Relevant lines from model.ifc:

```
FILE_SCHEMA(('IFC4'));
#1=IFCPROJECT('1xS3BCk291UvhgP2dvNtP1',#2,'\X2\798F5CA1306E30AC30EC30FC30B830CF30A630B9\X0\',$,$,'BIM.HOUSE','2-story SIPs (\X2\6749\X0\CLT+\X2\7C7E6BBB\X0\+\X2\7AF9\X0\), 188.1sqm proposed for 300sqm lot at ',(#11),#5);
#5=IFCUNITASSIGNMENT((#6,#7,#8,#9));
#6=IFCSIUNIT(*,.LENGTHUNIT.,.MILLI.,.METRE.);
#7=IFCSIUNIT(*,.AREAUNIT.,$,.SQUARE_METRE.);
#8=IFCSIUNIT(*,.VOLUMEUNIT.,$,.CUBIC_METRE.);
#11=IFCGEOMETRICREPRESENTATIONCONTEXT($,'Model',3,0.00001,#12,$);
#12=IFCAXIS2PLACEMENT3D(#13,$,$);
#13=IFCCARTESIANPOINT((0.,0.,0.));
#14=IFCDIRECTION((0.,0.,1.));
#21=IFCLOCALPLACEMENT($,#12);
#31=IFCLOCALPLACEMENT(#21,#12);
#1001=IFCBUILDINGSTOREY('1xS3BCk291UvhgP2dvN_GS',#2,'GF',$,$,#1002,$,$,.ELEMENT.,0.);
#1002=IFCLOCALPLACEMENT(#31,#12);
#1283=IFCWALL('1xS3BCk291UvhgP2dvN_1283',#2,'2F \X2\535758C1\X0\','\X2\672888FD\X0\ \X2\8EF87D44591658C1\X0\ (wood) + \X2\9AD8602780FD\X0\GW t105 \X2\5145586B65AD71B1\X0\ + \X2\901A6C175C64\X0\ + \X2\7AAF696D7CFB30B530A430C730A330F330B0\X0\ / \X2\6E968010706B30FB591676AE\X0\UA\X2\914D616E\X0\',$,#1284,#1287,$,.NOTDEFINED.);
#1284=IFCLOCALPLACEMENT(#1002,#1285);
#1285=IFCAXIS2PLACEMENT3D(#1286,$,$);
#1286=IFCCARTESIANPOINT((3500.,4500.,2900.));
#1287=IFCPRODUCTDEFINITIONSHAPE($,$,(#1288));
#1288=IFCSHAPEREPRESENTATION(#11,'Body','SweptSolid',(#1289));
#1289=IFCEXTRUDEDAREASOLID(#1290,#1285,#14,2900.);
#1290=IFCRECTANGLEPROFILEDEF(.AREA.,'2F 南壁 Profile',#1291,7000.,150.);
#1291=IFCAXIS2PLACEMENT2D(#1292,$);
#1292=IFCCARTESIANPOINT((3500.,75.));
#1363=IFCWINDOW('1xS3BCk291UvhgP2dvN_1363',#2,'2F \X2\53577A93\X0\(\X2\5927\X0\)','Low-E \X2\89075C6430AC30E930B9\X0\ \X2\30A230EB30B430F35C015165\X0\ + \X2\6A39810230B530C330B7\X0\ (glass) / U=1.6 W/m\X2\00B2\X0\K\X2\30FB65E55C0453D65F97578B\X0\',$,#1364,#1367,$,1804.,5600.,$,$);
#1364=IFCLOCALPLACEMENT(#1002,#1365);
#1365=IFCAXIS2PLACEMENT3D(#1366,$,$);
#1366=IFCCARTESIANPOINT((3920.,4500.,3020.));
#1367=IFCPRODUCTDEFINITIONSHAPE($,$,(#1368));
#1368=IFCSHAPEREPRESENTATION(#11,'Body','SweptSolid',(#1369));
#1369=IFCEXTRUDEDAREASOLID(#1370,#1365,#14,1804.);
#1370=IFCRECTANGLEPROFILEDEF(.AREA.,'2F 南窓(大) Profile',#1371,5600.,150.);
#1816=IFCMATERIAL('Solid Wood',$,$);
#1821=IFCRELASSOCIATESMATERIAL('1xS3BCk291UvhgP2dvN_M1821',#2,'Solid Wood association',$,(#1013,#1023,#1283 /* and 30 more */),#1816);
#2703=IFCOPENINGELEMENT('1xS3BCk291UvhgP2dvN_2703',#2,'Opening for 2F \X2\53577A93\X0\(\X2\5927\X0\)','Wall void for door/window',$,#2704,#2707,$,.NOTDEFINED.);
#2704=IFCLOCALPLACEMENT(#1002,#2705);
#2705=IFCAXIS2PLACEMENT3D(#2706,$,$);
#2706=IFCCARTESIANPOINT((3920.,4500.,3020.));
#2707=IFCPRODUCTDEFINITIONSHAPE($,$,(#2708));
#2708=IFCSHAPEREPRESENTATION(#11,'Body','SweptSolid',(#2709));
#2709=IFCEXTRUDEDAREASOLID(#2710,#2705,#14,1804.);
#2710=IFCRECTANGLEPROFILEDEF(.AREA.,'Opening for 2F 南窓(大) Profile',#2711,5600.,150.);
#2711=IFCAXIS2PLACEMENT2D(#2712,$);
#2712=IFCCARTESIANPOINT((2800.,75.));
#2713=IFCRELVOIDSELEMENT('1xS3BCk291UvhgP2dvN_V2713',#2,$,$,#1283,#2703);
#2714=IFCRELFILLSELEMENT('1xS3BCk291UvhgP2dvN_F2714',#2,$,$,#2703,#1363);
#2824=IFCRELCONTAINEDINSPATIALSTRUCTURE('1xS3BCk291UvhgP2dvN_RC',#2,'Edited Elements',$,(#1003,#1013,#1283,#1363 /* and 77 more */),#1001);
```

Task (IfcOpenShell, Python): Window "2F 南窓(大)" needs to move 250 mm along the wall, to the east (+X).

```python
import ifcopenshell
import ifcopenshell.api.geometry
import ifcopenshell.util.placement
import ifcopenshell.util.unit

model = ifcopenshell.open("model.ifc")
unit_scale = ifcopenshell.util.unit.calculate_unit_scale(model)

window = model.by_guid("1xS3BCk291UvhgP2dvN_1363")
opening = window.FillsVoids[0].RelatingOpeningElement
wall = opening.VoidsElements[0].RelatingBuildingElement

wall_matrix = ifcopenshell.util.placement.get_local_placement(wall.ObjectPlacement)
shift = wall_matrix[:3, 0] * 0.25 / unit_scale
before = ifcopenshell.util.placement.get_local_placement(window.ObjectPlacement)[:3, 3].copy()

# The window is not placed relative to its opening, so move both.
for product in (opening, window):
    matrix = ifcopenshell.util.placement.get_local_placement(product.ObjectPlacement)
    matrix[:3, 3] += shift
    ifcopenshell.api.geometry.edit_object_placement(model, product=product, matrix=matrix, is_si=False)

after = ifcopenshell.util.placement.get_local_placement(window.ObjectPlacement)[:3, 3]
print("window moved by", (after - before).round(3) + 0.0)

model.write("model_updated.ifc")
```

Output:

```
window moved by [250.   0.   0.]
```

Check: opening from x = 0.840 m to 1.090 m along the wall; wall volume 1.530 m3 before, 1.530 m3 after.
